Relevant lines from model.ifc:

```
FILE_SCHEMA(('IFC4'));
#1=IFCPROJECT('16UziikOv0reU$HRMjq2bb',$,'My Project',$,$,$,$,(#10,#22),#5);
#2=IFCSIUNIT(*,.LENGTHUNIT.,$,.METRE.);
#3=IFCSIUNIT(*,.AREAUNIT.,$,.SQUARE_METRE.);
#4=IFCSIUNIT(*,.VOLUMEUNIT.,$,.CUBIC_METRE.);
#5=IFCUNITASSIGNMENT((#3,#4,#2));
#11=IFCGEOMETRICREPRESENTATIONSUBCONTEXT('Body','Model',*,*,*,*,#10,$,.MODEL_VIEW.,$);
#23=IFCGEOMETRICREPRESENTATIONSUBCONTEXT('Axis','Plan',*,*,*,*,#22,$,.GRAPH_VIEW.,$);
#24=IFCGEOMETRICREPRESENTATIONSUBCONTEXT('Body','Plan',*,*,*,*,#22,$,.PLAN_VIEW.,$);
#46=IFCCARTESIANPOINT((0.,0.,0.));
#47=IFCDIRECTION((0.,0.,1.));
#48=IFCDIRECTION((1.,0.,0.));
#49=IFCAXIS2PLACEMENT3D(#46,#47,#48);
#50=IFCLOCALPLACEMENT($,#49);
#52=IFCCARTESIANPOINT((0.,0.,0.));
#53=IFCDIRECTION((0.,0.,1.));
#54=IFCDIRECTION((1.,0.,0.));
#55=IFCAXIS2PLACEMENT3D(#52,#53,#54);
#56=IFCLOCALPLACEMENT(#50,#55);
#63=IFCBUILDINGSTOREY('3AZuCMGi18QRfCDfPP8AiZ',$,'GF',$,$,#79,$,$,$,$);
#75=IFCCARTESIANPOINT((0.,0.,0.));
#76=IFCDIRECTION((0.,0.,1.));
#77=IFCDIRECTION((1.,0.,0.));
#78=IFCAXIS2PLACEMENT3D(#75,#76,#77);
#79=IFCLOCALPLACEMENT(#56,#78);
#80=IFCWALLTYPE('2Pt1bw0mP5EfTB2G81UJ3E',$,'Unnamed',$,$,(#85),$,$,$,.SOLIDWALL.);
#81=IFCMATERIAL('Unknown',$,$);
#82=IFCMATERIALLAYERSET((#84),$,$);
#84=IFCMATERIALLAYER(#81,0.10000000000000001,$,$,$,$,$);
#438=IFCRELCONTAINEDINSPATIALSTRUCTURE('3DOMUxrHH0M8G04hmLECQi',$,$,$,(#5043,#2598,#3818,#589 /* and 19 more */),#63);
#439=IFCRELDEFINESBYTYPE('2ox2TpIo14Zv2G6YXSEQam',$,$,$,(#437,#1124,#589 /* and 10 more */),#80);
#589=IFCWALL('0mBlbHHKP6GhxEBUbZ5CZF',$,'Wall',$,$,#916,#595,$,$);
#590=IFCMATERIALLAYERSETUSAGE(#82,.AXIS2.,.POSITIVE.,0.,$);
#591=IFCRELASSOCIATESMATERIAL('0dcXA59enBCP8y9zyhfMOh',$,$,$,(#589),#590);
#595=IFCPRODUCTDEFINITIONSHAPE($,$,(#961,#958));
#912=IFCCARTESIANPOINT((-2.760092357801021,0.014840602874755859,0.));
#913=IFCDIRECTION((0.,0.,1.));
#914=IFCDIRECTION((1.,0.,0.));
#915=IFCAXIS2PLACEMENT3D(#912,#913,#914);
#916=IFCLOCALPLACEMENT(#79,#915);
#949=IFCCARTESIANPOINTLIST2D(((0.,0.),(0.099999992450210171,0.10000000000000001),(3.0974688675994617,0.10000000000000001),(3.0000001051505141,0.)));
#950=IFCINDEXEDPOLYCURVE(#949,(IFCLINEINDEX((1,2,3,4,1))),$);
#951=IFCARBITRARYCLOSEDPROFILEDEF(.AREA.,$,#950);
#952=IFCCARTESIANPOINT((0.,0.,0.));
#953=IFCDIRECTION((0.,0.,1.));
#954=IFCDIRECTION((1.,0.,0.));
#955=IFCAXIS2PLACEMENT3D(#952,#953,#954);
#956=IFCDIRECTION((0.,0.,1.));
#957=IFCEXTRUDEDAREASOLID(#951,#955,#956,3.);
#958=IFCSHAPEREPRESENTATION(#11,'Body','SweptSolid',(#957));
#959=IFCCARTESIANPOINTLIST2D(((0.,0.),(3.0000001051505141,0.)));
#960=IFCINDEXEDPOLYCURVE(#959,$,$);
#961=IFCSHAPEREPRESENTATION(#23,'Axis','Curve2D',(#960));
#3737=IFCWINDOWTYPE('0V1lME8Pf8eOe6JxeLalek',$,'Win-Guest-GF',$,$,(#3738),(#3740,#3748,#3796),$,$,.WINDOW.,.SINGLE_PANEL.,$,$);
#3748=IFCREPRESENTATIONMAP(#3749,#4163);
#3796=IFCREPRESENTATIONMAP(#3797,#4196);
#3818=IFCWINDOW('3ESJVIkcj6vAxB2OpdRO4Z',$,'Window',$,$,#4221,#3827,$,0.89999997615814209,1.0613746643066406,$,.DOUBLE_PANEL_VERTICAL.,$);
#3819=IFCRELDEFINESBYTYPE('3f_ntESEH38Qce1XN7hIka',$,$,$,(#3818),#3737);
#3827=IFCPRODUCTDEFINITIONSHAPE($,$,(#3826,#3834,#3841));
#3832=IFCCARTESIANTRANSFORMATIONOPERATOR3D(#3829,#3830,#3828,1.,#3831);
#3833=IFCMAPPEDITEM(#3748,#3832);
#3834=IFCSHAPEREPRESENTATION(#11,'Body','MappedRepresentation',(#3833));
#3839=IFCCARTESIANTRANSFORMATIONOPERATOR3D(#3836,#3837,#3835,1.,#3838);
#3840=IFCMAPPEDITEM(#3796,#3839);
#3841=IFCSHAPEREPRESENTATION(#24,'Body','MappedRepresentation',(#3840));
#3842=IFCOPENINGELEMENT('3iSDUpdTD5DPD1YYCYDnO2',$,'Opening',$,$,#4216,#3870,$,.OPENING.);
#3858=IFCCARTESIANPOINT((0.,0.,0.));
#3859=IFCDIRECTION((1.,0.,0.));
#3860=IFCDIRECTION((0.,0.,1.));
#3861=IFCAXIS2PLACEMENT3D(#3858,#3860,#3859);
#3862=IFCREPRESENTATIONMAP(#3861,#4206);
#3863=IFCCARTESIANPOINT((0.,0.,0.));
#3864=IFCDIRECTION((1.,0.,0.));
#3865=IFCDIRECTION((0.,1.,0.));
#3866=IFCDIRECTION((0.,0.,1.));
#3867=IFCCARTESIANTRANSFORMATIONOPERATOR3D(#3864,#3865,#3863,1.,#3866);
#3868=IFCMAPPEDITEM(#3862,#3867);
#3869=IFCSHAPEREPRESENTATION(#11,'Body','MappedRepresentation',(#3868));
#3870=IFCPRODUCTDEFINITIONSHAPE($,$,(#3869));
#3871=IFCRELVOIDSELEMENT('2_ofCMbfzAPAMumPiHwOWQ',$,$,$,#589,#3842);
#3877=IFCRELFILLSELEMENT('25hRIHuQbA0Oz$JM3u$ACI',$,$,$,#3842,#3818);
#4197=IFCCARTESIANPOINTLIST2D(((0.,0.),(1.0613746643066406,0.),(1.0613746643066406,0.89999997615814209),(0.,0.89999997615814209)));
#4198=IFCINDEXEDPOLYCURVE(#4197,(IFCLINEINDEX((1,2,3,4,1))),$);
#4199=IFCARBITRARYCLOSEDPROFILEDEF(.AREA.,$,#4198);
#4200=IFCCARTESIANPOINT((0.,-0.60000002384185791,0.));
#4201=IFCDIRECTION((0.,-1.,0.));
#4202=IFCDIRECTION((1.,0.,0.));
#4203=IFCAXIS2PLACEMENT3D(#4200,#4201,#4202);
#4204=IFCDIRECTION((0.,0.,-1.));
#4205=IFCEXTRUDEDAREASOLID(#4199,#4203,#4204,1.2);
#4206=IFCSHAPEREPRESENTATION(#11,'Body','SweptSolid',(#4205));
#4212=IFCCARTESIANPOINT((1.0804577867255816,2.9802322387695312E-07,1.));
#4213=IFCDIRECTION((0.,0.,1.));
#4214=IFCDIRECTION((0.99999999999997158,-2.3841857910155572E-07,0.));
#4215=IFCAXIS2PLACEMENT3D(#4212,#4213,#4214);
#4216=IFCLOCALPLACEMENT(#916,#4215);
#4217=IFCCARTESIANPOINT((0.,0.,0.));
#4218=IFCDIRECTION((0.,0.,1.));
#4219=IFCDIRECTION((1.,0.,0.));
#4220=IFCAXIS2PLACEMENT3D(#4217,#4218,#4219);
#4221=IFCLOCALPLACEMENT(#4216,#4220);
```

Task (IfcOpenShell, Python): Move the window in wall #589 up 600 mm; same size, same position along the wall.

```python
import numpy as np
import ifcopenshell
import ifcopenshell.api.geometry
import ifcopenshell.util.placement
import ifcopenshell.util.unit

model = ifcopenshell.open("model.ifc")
unit_scale = ifcopenshell.util.unit.calculate_unit_scale(model)

window = model.by_guid("3ESJVIkcj6vAxB2OpdRO4Z")
opening = window.FillsVoids[0].RelatingOpeningElement
dz = 0.6 / unit_scale

shift = np.array([0.0, 0.0, dz])
# The window is placed relative to its opening, so it follows when the opening moves.
matrix = ifcopenshell.util.placement.get_local_placement(opening.ObjectPlacement)
matrix[:3, 3] += shift
ifcopenshell.api.geometry.edit_object_placement(
    model, product=opening, matrix=matrix, is_si=False, should_transform_children=True
)

print(f"moved by {dz * unit_scale:+.3f} m")

model.write("model_rev.ifc")
```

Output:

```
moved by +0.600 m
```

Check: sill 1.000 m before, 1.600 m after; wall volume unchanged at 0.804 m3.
